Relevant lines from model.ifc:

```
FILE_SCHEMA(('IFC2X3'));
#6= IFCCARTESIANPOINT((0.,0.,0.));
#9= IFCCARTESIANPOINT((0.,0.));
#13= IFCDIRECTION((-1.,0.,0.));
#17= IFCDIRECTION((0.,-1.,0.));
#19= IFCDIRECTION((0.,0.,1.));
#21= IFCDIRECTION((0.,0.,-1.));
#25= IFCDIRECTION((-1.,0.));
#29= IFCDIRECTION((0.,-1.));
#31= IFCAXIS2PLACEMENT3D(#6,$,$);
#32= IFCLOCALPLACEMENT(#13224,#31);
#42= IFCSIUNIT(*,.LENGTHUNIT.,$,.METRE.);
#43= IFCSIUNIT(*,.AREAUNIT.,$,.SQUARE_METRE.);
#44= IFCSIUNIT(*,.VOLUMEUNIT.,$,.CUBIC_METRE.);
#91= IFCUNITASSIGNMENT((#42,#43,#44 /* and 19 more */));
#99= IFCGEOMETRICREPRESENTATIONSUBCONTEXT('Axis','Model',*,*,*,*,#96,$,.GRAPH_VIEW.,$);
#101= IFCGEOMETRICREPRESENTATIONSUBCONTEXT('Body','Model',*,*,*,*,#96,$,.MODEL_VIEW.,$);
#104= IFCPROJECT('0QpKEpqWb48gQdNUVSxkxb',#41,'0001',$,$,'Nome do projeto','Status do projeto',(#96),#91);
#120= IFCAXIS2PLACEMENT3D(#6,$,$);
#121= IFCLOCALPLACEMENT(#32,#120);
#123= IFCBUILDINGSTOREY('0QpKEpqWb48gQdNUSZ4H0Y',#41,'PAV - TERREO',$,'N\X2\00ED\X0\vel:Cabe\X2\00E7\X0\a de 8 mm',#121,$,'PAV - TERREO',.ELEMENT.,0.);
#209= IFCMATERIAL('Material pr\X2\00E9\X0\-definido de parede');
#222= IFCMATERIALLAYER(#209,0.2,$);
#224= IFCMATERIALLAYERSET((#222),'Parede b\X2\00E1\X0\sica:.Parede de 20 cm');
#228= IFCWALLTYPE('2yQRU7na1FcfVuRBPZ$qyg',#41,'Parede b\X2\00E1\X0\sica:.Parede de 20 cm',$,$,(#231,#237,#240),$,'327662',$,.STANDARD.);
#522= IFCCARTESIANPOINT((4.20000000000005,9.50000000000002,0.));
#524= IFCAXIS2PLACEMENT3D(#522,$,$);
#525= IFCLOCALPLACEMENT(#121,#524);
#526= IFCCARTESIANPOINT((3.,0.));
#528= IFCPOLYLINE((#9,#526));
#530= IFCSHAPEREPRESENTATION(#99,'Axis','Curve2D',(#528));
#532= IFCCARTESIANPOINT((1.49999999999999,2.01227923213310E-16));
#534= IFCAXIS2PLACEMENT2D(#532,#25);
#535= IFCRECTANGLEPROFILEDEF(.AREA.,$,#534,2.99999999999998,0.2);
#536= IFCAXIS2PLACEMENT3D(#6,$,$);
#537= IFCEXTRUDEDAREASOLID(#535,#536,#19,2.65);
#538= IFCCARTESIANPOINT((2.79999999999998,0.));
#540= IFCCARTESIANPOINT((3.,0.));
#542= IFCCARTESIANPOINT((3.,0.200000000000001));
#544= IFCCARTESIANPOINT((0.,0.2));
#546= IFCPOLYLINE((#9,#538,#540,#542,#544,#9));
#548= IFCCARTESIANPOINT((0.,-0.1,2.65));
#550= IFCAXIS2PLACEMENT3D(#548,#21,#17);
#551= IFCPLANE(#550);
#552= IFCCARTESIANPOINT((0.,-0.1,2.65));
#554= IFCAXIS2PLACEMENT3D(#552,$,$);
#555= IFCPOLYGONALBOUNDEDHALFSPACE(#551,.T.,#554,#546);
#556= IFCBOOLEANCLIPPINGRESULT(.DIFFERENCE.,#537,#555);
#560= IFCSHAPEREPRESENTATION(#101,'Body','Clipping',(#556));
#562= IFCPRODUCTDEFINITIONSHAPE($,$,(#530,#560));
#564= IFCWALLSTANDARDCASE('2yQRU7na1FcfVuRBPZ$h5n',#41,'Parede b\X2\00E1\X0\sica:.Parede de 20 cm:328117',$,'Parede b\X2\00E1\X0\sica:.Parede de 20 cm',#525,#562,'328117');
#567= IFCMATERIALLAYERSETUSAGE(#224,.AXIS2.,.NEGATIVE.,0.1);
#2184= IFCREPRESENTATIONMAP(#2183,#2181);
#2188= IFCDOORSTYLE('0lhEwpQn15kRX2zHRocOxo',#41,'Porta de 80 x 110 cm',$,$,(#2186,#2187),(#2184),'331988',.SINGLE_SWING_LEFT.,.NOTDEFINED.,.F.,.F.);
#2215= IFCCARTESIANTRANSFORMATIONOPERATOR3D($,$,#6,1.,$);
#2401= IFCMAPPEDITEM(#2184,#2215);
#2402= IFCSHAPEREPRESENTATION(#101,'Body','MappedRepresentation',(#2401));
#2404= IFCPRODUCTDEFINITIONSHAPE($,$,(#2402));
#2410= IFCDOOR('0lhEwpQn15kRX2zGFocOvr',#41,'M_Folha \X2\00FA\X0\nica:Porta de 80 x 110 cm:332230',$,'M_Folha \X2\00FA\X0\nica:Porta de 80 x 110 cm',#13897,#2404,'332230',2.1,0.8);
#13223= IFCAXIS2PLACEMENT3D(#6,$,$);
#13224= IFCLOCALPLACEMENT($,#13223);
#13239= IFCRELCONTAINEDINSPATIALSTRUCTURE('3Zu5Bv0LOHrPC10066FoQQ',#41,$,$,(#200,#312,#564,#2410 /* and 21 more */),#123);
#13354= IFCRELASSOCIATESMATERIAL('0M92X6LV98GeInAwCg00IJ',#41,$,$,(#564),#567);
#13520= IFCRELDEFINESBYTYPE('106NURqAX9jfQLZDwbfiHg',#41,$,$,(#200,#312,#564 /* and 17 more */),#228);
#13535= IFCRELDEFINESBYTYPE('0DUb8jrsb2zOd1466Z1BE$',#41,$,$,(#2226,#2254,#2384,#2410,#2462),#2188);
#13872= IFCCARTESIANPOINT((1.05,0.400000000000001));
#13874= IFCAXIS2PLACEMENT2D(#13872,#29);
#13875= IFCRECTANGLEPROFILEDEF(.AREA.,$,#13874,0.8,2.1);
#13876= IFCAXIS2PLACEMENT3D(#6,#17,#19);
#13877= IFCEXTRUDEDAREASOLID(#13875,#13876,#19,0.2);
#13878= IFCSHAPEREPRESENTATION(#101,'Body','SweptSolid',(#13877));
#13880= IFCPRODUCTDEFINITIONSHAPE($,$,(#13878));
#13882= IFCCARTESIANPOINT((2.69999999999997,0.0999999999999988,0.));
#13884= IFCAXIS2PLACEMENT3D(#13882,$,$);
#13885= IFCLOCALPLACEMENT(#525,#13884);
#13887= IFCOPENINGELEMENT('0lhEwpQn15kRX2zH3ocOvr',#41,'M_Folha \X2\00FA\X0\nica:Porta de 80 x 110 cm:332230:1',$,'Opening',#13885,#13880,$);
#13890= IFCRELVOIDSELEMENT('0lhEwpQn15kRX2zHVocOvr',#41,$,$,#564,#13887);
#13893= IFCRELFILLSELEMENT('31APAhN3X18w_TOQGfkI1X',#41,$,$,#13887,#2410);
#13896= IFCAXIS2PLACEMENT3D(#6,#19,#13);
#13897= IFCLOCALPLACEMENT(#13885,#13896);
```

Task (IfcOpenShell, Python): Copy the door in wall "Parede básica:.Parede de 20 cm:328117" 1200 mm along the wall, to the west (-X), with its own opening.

```python
import ifcopenshell
import ifcopenshell.api.feature
import ifcopenshell.api.geometry
import ifcopenshell.api.root
import ifcopenshell.geom
import ifcopenshell.util.element
import ifcopenshell.util.placement
import ifcopenshell.util.shape
import ifcopenshell.util.unit

model = ifcopenshell.open("model.ifc")
unit_scale = ifcopenshell.util.unit.calculate_unit_scale(model)
settings = ifcopenshell.geom.settings()


def volume(element):
    """Net volume in cubic metres, openings subtracted."""
    shape = ifcopenshell.geom.create_shape(settings, element)
    return ifcopenshell.util.shape.get_volume(shape.geometry)


def reuse_history(source, copy):
    """copy_class also copies each property set's owner history, people and application; keep the originals."""
    for rel in copy.IsDefinedBy:
        if rel.is_a("IfcRelDefinesByProperties") and (history := rel.RelatingPropertyDefinition.OwnerHistory):
            rel.RelatingPropertyDefinition.OwnerHistory = source.OwnerHistory
            ifcopenshell.util.element.remove_deep2(model, history)


door = model.by_guid("0lhEwpQn15kRX2zGFocOvr")
opening = door.FillsVoids[0].RelatingOpeningElement
wall = opening.VoidsElements[0].RelatingBuildingElement
before = volume(wall)
shift = ifcopenshell.util.placement.get_local_placement(wall.ObjectPlacement)[:3, 0] * -1.2 / unit_scale

# copy_class copies the void relationship, type, container and properties, but no geometry.
new_opening = ifcopenshell.api.root.copy_class(model, product=opening)
new_opening.Representation = ifcopenshell.util.element.copy_deep(
    model, opening.Representation, exclude=["IfcGeometricRepresentationContext", "IfcRepresentationMap"]
)
new_opening.Name = "M_Folha única:Porta de 80 x 110 cm"
new_door = ifcopenshell.api.root.copy_class(model, product=door)
new_door.Representation = ifcopenshell.util.element.copy_deep(
    model, door.Representation, exclude=["IfcGeometricRepresentationContext", "IfcRepresentationMap"]
)
new_door.Name = "M_Folha única:Porta de 80 x 110 cm"
new_door.Tag = None
reuse_history(door, new_door)
fills = ifcopenshell.api.feature.add_filling(model, opening=new_opening, element=new_door)
fills.OwnerHistory = new_door.OwnerHistory  # required in IFC2X3

for old, new in ((opening, new_opening), (door, new_door)):
    matrix = ifcopenshell.util.placement.get_local_placement(old.ObjectPlacement)
    matrix[:3, 3] += shift
    ifcopenshell.api.geometry.edit_object_placement(model, product=new, matrix=matrix, is_si=False)

after = volume(wall)

print(f"wall volume {before:.3f} -> {after:.3f} m3")

model.write("model-out.ifc")
```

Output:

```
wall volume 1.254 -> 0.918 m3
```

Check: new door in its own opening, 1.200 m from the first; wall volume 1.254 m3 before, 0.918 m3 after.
